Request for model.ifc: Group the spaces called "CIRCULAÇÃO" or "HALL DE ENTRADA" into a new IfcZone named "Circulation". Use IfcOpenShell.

First a look at what the model holds.

```python
import ifcopenshell

model = ifcopenshell.open("model.ifc")
print(model.schema)
seen = {}
for space in model.by_type("IfcSpace"):
    seen[space.LongName] = seen.get(space.LongName, 0) + 1
for name, count in sorted(seen.items(), key=str):
    print(count, "x", name)
print("zones:", [z.Name for z in model.by_type("IfcZone")][:20])
```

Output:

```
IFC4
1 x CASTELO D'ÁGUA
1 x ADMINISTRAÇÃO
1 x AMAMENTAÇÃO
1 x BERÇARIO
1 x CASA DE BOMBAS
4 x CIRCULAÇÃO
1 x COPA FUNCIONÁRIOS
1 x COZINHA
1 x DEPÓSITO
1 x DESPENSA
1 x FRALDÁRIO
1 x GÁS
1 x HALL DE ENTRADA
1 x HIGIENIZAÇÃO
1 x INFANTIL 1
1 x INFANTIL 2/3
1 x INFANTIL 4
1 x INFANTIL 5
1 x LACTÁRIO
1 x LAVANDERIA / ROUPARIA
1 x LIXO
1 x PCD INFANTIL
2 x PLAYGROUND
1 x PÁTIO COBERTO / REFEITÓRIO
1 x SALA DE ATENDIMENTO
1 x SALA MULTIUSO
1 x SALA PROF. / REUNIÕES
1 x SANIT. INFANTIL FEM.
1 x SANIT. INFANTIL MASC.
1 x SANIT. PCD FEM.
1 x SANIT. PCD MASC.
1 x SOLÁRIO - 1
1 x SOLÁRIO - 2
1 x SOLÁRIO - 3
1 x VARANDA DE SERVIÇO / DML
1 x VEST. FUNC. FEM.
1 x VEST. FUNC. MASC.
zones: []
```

```python
import ifcopenshell
import ifcopenshell.api.group
import ifcopenshell.api.root

model = ifcopenshell.open("model.ifc")

names = {"CIRCULAÇÃO", "HALL DE ENTRADA"}
spaces = [s for s in model.by_type("IfcSpace") if s.LongName in names]

zone = ifcopenshell.api.root.create_entity(model, ifc_class="IfcZone", name="Circulation")
ifcopenshell.api.group.assign_group(model, products=spaces, group=zone)
print(len(spaces), "spaces in", zone.Name)

model.write("model_updated.ifc")
```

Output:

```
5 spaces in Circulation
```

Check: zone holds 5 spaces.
